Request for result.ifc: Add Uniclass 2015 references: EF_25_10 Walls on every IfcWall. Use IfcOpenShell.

First a look at what the model holds.

```python
import ifcopenshell

model = ifcopenshell.open("result.ifc")
print(model.schema)
print("classifications:", [c.Name for c in model.by_type("IfcClassification")])
for ifc_class in ("IfcDoor", "IfcRoof", "IfcStair", "IfcWall", "IfcWindow"):
    print(ifc_class, len(model.by_type(ifc_class)))
```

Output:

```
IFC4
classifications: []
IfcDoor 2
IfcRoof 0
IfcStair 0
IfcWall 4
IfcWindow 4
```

```python
import ifcopenshell
import ifcopenshell.api.classification

model = ifcopenshell.open("result.ifc")

system = ifcopenshell.api.classification.add_classification(model, classification="Uniclass 2015")

codes = {
    "IfcWall": ("EF_25_10", "Walls"),
}
for ifc_class, (code, name) in codes.items():
    products = model.by_type(ifc_class)
    ifcopenshell.api.classification.add_reference(
        model, products=products, classification=system, identification=code, name=name
    )
    print(code, len(products))

model.write("result_updated.ifc")
```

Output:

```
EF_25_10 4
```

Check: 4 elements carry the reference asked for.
